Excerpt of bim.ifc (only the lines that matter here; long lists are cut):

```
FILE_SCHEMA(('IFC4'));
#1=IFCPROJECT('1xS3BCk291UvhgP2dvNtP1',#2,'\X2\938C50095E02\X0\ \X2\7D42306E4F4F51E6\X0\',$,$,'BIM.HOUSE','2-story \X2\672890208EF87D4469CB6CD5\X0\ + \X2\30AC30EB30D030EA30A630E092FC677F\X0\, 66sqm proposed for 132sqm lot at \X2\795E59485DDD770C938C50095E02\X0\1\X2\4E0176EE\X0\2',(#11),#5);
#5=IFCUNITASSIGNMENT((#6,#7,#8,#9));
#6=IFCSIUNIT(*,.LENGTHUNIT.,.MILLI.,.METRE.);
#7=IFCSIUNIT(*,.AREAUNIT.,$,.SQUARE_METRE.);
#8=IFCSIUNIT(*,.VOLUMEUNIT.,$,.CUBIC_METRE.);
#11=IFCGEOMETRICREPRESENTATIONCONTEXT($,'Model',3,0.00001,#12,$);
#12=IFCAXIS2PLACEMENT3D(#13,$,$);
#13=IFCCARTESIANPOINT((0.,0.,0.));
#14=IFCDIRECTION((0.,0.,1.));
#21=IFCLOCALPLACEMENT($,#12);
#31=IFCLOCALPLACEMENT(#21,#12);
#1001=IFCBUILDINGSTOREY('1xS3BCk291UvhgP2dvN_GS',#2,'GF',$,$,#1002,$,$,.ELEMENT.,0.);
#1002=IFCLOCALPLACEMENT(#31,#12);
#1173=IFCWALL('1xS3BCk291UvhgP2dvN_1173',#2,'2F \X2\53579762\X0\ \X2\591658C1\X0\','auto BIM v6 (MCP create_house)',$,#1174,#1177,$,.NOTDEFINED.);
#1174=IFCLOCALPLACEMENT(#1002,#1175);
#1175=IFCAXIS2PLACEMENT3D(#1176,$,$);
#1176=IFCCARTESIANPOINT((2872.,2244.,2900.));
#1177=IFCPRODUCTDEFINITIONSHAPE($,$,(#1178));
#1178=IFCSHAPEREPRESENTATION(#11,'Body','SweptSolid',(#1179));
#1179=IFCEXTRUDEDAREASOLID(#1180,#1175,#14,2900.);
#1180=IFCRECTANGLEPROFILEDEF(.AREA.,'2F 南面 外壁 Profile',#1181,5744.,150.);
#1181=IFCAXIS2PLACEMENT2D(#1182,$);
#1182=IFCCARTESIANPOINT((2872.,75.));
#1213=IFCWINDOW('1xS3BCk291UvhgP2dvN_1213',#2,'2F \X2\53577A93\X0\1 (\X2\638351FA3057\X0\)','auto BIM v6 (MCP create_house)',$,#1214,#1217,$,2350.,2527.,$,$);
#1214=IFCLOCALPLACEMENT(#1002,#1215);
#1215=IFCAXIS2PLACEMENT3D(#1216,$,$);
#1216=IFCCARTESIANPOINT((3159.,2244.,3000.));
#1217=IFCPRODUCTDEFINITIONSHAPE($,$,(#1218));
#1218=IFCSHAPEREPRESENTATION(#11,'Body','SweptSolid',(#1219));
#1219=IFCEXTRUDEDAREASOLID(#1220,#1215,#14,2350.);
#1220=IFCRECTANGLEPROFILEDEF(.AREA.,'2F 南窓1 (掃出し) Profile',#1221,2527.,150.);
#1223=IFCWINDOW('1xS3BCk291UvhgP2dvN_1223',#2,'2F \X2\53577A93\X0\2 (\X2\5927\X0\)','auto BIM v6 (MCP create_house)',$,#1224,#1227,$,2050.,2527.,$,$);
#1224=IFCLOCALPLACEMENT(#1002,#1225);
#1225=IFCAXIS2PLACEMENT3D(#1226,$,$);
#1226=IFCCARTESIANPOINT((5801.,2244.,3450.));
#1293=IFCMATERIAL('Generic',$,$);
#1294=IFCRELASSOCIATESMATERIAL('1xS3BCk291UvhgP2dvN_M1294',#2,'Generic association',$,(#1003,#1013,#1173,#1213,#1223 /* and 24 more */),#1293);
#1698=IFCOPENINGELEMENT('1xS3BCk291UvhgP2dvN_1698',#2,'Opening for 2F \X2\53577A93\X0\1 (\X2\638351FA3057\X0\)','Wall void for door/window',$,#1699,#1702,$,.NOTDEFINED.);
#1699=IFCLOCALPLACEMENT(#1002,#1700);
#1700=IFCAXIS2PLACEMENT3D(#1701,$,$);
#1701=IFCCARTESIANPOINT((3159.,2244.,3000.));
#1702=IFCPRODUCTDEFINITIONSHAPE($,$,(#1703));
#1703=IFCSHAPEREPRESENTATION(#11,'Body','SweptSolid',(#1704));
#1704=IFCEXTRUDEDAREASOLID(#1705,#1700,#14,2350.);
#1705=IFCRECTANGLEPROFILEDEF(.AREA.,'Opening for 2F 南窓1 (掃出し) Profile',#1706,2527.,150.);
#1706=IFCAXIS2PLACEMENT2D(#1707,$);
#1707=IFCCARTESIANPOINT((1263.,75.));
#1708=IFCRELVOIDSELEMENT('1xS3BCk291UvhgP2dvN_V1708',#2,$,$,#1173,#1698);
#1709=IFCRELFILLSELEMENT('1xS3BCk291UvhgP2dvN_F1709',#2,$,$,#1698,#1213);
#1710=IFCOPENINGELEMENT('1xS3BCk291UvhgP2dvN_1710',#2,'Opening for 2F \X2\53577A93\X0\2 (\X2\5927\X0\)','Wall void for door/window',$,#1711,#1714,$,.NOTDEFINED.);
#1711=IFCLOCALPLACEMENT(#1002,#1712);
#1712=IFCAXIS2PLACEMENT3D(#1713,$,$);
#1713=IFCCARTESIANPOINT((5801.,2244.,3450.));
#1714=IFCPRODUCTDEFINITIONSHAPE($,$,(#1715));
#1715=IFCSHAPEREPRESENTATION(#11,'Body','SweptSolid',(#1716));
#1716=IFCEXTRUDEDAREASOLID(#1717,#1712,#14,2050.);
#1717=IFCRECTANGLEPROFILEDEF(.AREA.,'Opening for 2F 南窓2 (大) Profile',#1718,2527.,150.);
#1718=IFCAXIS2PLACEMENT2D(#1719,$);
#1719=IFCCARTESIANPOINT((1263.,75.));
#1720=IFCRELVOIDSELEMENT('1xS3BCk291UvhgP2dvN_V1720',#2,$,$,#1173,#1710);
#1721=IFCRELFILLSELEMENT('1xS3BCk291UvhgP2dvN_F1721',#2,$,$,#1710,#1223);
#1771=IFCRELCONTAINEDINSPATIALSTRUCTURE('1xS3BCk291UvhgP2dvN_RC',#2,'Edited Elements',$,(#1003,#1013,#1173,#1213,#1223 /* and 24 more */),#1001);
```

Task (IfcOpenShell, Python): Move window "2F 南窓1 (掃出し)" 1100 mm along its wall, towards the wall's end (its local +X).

```python
import ifcopenshell
import ifcopenshell.api.geometry
import ifcopenshell.util.placement
import ifcopenshell.util.unit

model = ifcopenshell.open("bim.ifc")
unit_scale = ifcopenshell.util.unit.calculate_unit_scale(model)

window = model.by_id(1213)
opening = window.FillsVoids[0].RelatingOpeningElement
wall = opening.VoidsElements[0].RelatingBuildingElement

wall_matrix = ifcopenshell.util.placement.get_local_placement(wall.ObjectPlacement)
shift = wall_matrix[:3, 0] * 1.1 / unit_scale
before = ifcopenshell.util.placement.get_local_placement(window.ObjectPlacement)[:3, 3].copy()

# The window is not placed relative to its opening, so move both.
for product in (opening, window):
    matrix = ifcopenshell.util.placement.get_local_placement(product.ObjectPlacement)
    matrix[:3, 3] += shift
    ifcopenshell.api.geometry.edit_object_placement(model, product=product, matrix=matrix, is_si=False)

after = ifcopenshell.util.placement.get_local_placement(window.ObjectPlacement)[:3, 3]
print("window moved by", (after - before).round(3) + 0.0)

model.write("bim-out.ifc")
```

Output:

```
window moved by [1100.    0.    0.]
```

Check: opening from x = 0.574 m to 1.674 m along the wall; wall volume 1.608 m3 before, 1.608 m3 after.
